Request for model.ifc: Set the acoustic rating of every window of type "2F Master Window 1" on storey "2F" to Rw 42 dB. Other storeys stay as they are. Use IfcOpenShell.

First a look at what the model holds.

```python
import ifcopenshell
import ifcopenshell.util.element

model = ifcopenshell.open("model.ifc")
print(model.schema)
storey = next(s for s in model.by_type("IfcBuildingStorey") if s.Name == "2F")
windows = [e for e in ifcopenshell.util.element.get_decomposition(storey) if e.is_a("IfcWindow")]
seen = {}
for e in windows:
    element_type = ifcopenshell.util.element.get_type(e)
    key = (element_type.Name if element_type != e and element_type else None, ifcopenshell.util.element.get_pset(e, "Pset_WindowCommon", "AcousticRating"))
    seen[key] = seen.get(key, 0) + 1
for (name, value), count in sorted(seen.items(), key=str):
    print(count, "x", name, "|", value)
```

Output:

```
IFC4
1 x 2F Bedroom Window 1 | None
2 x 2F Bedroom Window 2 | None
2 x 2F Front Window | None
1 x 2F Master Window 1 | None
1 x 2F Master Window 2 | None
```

```python
import ifcopenshell
import ifcopenshell.api.pset
import ifcopenshell.util.element

model = ifcopenshell.open("model.ifc")

storey = next(s for s in model.by_type("IfcBuildingStorey") if s.Name == "2F")
windows = [e for e in ifcopenshell.util.element.get_decomposition(storey) if e.is_a("IfcWindow")]

count = 0
for e in windows:
    element_type = ifcopenshell.util.element.get_type(e)
    if element_type in (None, e) or element_type.Name != "2F Master Window 1":
        continue
    # add_pset returns the element's existing set when there is one.
    pset = ifcopenshell.api.pset.add_pset(model, product=e, name="Pset_WindowCommon")
    ifcopenshell.api.pset.edit_pset(model, pset=pset, properties={"AcousticRating": "Rw 42 dB"})
    count += 1

print(count, "windows updated")

model.write("model_edited.ifc")
```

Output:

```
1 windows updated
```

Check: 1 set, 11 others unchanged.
